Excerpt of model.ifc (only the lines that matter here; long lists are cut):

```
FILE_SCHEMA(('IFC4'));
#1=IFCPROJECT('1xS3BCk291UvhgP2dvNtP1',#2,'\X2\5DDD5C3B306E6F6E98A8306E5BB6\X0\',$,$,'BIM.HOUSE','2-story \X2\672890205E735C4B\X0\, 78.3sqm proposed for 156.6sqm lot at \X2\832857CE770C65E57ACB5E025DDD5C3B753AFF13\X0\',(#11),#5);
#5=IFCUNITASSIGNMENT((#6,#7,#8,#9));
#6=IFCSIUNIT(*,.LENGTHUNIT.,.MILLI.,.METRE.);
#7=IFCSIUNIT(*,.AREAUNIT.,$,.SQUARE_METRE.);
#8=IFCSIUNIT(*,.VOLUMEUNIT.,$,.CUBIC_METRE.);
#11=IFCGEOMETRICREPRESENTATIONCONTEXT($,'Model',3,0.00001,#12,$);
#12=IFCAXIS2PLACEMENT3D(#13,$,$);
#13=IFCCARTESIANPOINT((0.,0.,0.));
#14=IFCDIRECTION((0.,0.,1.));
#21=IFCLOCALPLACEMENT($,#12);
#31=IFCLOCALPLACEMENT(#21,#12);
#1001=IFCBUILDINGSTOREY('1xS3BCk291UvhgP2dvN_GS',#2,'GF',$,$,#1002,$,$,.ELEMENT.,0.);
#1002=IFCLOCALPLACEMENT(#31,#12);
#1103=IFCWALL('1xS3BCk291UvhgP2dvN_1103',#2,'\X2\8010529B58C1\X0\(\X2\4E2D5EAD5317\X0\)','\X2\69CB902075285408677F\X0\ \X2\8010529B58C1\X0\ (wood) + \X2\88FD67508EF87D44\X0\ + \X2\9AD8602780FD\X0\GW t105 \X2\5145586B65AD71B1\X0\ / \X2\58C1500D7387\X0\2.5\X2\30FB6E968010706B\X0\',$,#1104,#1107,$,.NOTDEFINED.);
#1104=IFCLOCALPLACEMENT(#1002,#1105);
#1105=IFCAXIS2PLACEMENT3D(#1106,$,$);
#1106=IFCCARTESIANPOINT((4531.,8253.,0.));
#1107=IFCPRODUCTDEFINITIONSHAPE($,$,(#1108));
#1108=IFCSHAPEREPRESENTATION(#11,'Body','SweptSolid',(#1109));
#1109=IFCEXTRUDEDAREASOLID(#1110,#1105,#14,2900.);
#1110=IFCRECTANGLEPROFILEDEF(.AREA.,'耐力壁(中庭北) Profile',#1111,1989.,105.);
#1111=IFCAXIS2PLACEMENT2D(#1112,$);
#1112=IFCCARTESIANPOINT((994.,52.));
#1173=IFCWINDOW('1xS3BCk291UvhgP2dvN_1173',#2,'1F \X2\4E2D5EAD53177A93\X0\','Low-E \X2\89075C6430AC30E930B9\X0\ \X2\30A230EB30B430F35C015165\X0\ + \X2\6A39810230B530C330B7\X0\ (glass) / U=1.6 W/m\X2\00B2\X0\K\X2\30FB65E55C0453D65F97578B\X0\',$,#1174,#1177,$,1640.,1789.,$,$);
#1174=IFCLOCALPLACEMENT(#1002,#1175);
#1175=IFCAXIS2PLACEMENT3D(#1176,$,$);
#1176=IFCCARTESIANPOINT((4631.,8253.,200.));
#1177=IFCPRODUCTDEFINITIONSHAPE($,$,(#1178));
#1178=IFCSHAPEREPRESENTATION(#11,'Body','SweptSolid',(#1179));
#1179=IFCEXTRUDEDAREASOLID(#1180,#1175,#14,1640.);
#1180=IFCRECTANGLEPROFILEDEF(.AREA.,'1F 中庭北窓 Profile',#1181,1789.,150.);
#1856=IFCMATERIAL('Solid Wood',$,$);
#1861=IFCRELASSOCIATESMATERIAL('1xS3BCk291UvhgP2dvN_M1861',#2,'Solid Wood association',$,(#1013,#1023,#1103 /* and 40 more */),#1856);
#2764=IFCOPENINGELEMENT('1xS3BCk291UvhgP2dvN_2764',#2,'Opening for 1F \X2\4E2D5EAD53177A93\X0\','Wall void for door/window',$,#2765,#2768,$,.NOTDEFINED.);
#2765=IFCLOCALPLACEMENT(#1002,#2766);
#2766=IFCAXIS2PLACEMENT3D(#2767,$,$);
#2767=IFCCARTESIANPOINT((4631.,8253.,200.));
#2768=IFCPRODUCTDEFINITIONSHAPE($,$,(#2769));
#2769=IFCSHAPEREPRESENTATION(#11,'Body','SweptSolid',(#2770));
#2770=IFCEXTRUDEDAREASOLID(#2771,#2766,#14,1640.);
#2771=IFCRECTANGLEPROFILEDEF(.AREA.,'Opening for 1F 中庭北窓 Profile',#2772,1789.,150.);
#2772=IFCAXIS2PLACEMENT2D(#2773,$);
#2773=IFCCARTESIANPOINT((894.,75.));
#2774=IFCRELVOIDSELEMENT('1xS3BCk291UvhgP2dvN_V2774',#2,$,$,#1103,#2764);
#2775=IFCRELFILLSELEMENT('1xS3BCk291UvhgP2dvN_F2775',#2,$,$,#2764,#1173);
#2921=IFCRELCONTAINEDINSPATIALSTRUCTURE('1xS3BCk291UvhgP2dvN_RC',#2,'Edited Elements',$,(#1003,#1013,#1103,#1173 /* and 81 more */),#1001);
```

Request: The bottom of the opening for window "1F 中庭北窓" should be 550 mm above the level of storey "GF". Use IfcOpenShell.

```python
import numpy as np
import ifcopenshell
import ifcopenshell.api.geometry
import ifcopenshell.geom
import ifcopenshell.util.element
import ifcopenshell.util.placement
import ifcopenshell.util.shape
import ifcopenshell.util.unit

model = ifcopenshell.open("model.ifc")
unit_scale = ifcopenshell.util.unit.calculate_unit_scale(model)

window = model.by_id(1173)
opening = window.FillsVoids[0].RelatingOpeningElement
storey = ifcopenshell.util.element.get_container(window, ifc_class="IfcBuildingStorey")
level = ifcopenshell.util.placement.get_local_placement(storey.ObjectPlacement)[2, 3]

# The opening's origin need not be at the sill, so measure its lowest point.
shape = ifcopenshell.geom.create_shape(ifcopenshell.geom.settings(), opening)
bottom = ifcopenshell.util.shape.get_shape_bottom_elevation(shape, shape.geometry) / unit_scale
dz = level + 0.55 / unit_scale - bottom

shift = np.array([0.0, 0.0, dz])
# The window is not placed relative to its opening, so move both.
for product in (opening, window):
    matrix = ifcopenshell.util.placement.get_local_placement(product.ObjectPlacement)
    matrix[:3, 3] += shift
    ifcopenshell.api.geometry.edit_object_placement(model, product=product, matrix=matrix, is_si=False)

print(f"moved by {dz * unit_scale:+.3f} m")

model.write("model_updated.ifc")
```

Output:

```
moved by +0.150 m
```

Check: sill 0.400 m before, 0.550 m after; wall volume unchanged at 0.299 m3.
